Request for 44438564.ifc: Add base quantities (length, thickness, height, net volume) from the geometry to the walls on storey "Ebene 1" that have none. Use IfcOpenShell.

First a look at what the model holds.

```python
import ifcopenshell
import ifcopenshell.util.element
import ifcopenshell.util.unit

model = ifcopenshell.open("44438564.ifc")
print(model.schema)
for unit_type in ("LENGTHUNIT", "AREAUNIT", "VOLUMEUNIT"):
    print(unit_type, ifcopenshell.util.unit.calculate_unit_scale(model, unit_type))
storey = next(s for s in model.by_type("IfcBuildingStorey") if s.Name == "Ebene 1")
walls = [e for e in ifcopenshell.util.element.get_decomposition(storey) if e.is_a("IfcWall")]
for e in sorted(walls, key=lambda e: e.id()):
    print(e.id(), e.is_a(), e.Name, list(ifcopenshell.util.element.get_psets(e, qtos_only=True)), sep=" | ")
```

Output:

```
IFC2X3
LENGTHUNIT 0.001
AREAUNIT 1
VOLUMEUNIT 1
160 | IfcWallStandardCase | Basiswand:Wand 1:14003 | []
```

```python
import ifcopenshell
import ifcopenshell.api.pset
import ifcopenshell.geom
import ifcopenshell.util.element
import ifcopenshell.util.shape
import ifcopenshell.util.unit

model = ifcopenshell.open("44438564.ifc")
unit_scale = ifcopenshell.util.unit.calculate_unit_scale(model)
volume_scale = ifcopenshell.util.unit.calculate_unit_scale(model, "VOLUMEUNIT")
settings = ifcopenshell.geom.settings()

storey = next(s for s in model.by_type("IfcBuildingStorey") if s.Name == "Ebene 1")
walls = [e for e in ifcopenshell.util.element.get_decomposition(storey) if e.is_a("IfcWall")]

for e in sorted(walls, key=lambda e: e.id()):
    if ifcopenshell.util.element.get_psets(e, qtos_only=True, should_inherit=False):
        continue
    # Geometry comes back in metres, in the element's own axes.
    shape = ifcopenshell.geom.create_shape(settings, e)
    values = {
        "Length": ifcopenshell.util.shape.get_x(shape.geometry) / unit_scale,
        "Width": ifcopenshell.util.shape.get_y(shape.geometry) / unit_scale,
        "Height": ifcopenshell.util.shape.get_z(shape.geometry) / unit_scale,
        "NetVolume": ifcopenshell.util.shape.get_volume(shape.geometry) / volume_scale,
    }
    qto = ifcopenshell.api.pset.add_qto(model, product=e, name="BaseQuantities")
    ifcopenshell.api.pset.edit_qto(model, qto=qto, properties=values)
    print(e.id(), {k: round(v, 3) for k, v in values.items()})

model.write("44438564_edited.ifc")
```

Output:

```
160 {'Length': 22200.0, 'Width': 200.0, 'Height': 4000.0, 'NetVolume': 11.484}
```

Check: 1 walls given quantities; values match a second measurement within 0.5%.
